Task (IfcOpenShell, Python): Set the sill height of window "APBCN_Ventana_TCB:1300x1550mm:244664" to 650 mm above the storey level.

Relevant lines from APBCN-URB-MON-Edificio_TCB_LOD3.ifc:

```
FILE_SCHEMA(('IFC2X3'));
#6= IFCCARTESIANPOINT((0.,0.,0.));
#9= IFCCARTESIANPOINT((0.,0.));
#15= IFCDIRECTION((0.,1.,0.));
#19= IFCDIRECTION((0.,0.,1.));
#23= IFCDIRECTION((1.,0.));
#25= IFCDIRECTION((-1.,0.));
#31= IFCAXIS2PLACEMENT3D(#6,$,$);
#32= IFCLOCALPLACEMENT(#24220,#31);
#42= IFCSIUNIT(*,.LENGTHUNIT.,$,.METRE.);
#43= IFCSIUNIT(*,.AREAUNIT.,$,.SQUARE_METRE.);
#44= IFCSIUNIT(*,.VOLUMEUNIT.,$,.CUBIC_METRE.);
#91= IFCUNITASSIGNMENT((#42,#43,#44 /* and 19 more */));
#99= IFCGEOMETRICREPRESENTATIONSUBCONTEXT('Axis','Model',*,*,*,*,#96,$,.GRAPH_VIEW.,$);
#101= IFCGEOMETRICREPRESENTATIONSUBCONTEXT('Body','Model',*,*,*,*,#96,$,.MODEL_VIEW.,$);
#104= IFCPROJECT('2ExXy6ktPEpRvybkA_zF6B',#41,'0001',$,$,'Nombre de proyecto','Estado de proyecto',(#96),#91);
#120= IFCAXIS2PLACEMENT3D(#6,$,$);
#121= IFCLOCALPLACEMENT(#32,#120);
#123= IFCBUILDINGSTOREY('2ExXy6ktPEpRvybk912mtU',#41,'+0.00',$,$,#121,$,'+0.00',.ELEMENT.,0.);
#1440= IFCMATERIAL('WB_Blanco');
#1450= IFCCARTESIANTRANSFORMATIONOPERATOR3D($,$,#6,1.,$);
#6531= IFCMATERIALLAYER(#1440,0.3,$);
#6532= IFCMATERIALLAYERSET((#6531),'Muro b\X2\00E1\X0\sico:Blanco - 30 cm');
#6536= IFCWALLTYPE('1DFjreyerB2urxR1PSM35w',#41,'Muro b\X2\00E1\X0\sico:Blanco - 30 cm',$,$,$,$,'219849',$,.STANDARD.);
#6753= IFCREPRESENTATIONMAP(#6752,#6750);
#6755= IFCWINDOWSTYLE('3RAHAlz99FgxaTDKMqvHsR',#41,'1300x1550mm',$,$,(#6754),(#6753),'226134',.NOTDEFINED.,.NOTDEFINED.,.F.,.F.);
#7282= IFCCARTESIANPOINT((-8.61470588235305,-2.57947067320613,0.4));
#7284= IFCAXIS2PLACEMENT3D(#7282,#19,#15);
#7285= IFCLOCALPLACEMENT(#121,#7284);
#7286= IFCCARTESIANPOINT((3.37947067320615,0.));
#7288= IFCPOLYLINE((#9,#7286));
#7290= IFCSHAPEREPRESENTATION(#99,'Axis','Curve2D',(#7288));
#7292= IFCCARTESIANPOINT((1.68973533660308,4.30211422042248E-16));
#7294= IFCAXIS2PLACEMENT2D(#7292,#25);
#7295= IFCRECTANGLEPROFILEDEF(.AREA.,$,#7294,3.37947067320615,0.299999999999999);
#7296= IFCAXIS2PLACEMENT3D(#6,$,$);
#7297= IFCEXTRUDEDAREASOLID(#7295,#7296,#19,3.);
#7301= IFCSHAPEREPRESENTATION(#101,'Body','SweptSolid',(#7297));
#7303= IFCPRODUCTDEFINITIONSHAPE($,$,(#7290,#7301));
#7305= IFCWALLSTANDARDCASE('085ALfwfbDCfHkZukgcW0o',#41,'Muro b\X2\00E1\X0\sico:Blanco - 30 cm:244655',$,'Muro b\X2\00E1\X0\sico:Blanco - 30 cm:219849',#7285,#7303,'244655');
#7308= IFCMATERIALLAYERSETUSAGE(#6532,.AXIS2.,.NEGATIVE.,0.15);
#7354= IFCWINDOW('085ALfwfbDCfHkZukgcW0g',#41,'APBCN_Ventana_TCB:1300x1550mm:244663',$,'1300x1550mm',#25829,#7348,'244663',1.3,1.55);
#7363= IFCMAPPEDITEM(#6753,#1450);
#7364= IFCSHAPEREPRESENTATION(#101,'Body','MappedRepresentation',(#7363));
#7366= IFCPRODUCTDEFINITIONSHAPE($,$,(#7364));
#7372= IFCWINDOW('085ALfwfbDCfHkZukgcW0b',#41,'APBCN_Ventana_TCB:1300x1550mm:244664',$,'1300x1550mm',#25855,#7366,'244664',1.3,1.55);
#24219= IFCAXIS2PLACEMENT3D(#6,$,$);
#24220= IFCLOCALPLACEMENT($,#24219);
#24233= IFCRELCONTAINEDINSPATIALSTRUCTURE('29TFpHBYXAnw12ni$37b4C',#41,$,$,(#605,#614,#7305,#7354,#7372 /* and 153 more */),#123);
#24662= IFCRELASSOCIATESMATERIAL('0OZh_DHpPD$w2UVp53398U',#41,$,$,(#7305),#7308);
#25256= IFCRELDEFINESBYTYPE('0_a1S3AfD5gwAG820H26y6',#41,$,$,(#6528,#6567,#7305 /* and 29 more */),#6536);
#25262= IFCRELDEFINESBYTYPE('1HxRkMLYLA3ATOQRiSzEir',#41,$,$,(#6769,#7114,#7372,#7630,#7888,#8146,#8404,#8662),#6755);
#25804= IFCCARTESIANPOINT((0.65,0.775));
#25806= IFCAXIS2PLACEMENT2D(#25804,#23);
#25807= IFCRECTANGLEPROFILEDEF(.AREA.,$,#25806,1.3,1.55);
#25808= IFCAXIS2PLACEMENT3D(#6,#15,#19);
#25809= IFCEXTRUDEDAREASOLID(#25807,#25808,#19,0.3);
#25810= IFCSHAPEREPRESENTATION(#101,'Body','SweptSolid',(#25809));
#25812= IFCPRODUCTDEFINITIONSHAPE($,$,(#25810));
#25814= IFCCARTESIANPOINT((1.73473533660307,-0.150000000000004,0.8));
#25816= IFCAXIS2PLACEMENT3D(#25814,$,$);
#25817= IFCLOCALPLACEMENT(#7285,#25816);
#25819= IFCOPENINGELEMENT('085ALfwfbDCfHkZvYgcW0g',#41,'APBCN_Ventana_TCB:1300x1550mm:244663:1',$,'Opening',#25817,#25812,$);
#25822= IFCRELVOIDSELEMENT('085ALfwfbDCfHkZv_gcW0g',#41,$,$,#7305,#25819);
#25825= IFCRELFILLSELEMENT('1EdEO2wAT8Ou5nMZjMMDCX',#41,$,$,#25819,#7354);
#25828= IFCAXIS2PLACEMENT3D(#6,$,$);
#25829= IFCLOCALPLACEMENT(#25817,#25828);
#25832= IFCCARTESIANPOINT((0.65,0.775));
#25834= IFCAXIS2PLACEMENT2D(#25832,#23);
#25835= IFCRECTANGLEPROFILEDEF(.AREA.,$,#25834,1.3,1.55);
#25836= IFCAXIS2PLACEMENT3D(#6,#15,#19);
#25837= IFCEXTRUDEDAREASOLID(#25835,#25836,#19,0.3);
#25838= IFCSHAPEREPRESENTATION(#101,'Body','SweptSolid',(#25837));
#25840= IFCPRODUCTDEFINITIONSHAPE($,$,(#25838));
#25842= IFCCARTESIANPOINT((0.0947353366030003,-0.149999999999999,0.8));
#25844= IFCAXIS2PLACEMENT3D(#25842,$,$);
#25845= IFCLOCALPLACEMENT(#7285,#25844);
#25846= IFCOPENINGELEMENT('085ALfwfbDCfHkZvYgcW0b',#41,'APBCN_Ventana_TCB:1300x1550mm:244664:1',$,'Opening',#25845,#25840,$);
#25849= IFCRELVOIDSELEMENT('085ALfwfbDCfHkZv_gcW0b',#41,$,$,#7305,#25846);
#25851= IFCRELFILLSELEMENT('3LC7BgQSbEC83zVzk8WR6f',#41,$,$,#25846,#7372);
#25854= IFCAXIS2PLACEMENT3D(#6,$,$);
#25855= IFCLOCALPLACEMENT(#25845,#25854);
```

```python
import numpy as np
import ifcopenshell
import ifcopenshell.api.geometry
import ifcopenshell.geom
import ifcopenshell.util.element
import ifcopenshell.util.placement
import ifcopenshell.util.shape
import ifcopenshell.util.unit

model = ifcopenshell.open("APBCN-URB-MON-Edificio_TCB_LOD3.ifc")
unit_scale = ifcopenshell.util.unit.calculate_unit_scale(model)

window = model.by_guid("085ALfwfbDCfHkZukgcW0b")
opening = window.FillsVoids[0].RelatingOpeningElement
storey = ifcopenshell.util.element.get_container(window, ifc_class="IfcBuildingStorey")
level = ifcopenshell.util.placement.get_local_placement(storey.ObjectPlacement)[2, 3]

# The opening's origin need not be at the sill, so measure its lowest point.
shape = ifcopenshell.geom.create_shape(ifcopenshell.geom.settings(), opening)
bottom = ifcopenshell.util.shape.get_shape_bottom_elevation(shape, shape.geometry) / unit_scale
dz = level + 0.65 / unit_scale - bottom

shift = np.array([0.0, 0.0, dz])
# The window is placed relative to its opening, so it follows when the opening moves.
matrix = ifcopenshell.util.placement.get_local_placement(opening.ObjectPlacement)
matrix[:3, 3] += shift
ifcopenshell.api.geometry.edit_object_placement(
    model, product=opening, matrix=matrix, is_si=False, should_transform_children=True
)

print(f"moved by {dz * unit_scale:+.3f} m")

model.write("APBCN-URB-MON-Edificio_TCB_LOD3_edited.ifc")
```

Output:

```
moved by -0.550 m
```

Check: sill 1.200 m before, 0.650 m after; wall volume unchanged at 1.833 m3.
